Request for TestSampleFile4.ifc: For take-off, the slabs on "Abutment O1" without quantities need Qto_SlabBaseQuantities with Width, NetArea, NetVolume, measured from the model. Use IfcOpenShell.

First a look at what the model holds.

```python
import ifcopenshell
import ifcopenshell.util.element
import ifcopenshell.util.unit

model = ifcopenshell.open("TestSampleFile4.ifc")
print(model.schema)
for unit_type in ("LENGTHUNIT", "AREAUNIT", "VOLUMEUNIT"):
    print(unit_type, ifcopenshell.util.unit.calculate_unit_scale(model, unit_type))
storey = next(s for s in model.by_type("IfcBuildingStorey") if s.Name == "Abutment O1")
slabs = [e for e in ifcopenshell.util.element.get_decomposition(storey) if e.is_a("IfcSlab")]
for e in sorted(slabs, key=lambda e: e.id()):
    print(e.id(), e.is_a(), e.Name, list(ifcopenshell.util.element.get_psets(e, qtos_only=True)), sep=" | ")
```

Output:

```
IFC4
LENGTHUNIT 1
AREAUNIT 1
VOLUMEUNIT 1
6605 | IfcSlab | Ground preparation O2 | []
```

```python
import ifcopenshell
import ifcopenshell.api.pset
import ifcopenshell.geom
import ifcopenshell.util.element
import ifcopenshell.util.shape
import ifcopenshell.util.unit

model = ifcopenshell.open("TestSampleFile4.ifc")
unit_scale = ifcopenshell.util.unit.calculate_unit_scale(model)
area_scale = ifcopenshell.util.unit.calculate_unit_scale(model, "AREAUNIT")
volume_scale = ifcopenshell.util.unit.calculate_unit_scale(model, "VOLUMEUNIT")
settings = ifcopenshell.geom.settings()

storey = next(s for s in model.by_type("IfcBuildingStorey") if s.Name == "Abutment O1")
slabs = [e for e in ifcopenshell.util.element.get_decomposition(storey) if e.is_a("IfcSlab")]

for e in sorted(slabs, key=lambda e: e.id()):
    if ifcopenshell.util.element.get_psets(e, qtos_only=True, should_inherit=False):
        continue
    # Geometry comes back in metres, in the element's own axes.
    shape = ifcopenshell.geom.create_shape(settings, e)
    values = {
        "Width": ifcopenshell.util.shape.get_z(shape.geometry) / unit_scale,
        "NetArea": ifcopenshell.util.shape.get_footprint_area(shape.geometry) / area_scale,
        "NetVolume": ifcopenshell.util.shape.get_volume(shape.geometry) / volume_scale,
    }
    qto = ifcopenshell.api.pset.add_qto(model, product=e, name="Qto_SlabBaseQuantities")
    ifcopenshell.api.pset.edit_qto(model, qto=qto, properties=values)
    print(e.id(), {k: round(v, 3) for k, v in values.items()})

model.write("TestSampleFile4_updated.ifc")
```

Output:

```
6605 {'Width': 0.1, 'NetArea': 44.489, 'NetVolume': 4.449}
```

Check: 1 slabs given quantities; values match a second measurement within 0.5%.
